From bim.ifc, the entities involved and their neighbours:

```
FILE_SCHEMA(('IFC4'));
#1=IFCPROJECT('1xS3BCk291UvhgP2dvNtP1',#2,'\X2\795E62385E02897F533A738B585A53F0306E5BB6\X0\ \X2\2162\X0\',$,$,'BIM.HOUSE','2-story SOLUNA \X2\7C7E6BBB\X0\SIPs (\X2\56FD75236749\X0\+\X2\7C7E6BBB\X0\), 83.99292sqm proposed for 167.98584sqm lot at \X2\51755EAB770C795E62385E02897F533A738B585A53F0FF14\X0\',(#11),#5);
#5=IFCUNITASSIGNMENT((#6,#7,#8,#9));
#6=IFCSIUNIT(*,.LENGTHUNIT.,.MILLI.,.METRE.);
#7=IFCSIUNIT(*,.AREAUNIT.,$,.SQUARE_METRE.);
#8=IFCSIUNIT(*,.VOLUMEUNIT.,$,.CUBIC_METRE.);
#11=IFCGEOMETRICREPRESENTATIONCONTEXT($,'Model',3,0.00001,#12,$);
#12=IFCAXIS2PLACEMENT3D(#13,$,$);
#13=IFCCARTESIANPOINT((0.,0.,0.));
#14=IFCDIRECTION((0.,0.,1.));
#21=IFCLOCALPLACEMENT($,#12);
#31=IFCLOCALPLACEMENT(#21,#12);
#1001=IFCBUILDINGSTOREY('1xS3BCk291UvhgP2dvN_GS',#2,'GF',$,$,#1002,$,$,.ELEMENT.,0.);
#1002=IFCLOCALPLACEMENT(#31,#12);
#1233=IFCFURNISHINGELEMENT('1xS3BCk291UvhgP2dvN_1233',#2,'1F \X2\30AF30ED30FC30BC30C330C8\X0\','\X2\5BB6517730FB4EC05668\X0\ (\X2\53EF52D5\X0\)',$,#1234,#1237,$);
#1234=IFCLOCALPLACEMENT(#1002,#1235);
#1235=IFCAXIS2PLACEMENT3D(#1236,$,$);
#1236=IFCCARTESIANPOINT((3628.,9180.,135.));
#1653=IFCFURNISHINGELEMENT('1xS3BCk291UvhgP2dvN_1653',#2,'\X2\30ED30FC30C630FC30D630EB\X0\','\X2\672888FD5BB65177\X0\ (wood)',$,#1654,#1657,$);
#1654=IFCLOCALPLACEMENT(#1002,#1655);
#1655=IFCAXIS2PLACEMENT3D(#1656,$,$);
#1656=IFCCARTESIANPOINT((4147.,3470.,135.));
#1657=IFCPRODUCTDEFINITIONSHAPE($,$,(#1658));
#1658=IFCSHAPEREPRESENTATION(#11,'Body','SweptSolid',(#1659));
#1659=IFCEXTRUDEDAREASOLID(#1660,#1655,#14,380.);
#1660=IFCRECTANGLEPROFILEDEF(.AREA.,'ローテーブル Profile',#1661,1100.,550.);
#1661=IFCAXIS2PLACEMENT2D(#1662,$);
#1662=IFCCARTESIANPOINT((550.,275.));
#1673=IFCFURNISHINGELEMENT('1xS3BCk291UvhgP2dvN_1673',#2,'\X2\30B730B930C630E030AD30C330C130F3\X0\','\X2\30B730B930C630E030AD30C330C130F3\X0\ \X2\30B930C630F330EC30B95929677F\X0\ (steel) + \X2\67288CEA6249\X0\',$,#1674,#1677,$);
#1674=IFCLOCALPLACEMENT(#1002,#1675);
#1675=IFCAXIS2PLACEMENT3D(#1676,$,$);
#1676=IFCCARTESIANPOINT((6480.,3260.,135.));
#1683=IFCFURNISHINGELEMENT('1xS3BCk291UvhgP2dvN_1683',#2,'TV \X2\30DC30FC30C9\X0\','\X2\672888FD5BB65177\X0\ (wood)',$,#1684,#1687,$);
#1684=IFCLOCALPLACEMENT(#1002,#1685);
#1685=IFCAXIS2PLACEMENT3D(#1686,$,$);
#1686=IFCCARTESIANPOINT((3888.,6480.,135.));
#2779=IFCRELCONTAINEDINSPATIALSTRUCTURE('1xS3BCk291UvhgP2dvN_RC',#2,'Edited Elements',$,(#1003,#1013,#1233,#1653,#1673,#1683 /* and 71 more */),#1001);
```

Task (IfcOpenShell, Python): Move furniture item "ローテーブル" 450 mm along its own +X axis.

```python
import ifcopenshell
import ifcopenshell.api.geometry
import ifcopenshell.util.placement

model = ifcopenshell.open("bim.ifc")

item = model.by_guid("1xS3BCk291UvhgP2dvN_1653")
matrix = ifcopenshell.util.placement.get_local_placement(item.ObjectPlacement)
matrix[:3, 3] += matrix[:3, 0] * 450.0
ifcopenshell.api.geometry.edit_object_placement(model, product=item, matrix=matrix, is_si=False)

print(ifcopenshell.util.placement.get_local_placement(item.ObjectPlacement).round(3) + 0.0)

model.write("bim-out.ifc")
```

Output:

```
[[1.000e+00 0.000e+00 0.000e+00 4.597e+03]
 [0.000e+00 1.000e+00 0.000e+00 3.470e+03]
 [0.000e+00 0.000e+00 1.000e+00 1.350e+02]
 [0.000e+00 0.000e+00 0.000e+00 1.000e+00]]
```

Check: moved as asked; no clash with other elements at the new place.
